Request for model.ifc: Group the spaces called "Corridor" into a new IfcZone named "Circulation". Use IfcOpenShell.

First a look at what the model holds.

```python
import ifcopenshell

model = ifcopenshell.open("model.ifc")
print(model.schema)
seen = {}
for space in model.by_type("IfcSpace"):
    seen[space.LongName] = seen.get(space.LongName, 0) + 1
for name, count in sorted(seen.items(), key=str):
    print(count, "x", name)
print("zones:", [z.Name for z in model.by_type("IfcZone")][:20])
```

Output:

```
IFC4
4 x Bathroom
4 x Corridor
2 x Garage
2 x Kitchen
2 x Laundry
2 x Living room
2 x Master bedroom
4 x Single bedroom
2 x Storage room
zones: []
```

```python
import ifcopenshell
import ifcopenshell.api.group
import ifcopenshell.api.root

model = ifcopenshell.open("model.ifc")

names = {"Corridor"}
spaces = [s for s in model.by_type("IfcSpace") if s.LongName in names]

zone = ifcopenshell.api.root.create_entity(model, ifc_class="IfcZone", name="Circulation")
ifcopenshell.api.group.assign_group(model, products=spaces, group=zone)
print(len(spaces), "spaces in", zone.Name)

model.write("model-out.ifc")
```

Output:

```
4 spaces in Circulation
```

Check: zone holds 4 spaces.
